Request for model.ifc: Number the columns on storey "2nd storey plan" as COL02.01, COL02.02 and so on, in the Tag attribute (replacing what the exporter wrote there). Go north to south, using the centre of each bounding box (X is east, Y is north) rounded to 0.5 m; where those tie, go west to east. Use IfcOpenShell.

First a look at what the model holds.

```python
import ifcopenshell
import ifcopenshell.util.element
import ifcopenshell.util.placement

model = ifcopenshell.open("model.ifc")
print(model.schema)
storey = next(s for s in model.by_type("IfcBuildingStorey") if s.Name == "2nd storey plan")
columns = [e for e in ifcopenshell.util.element.get_decomposition(storey) if e.is_a("IfcColumn")]
for e in sorted(columns, key=lambda e: e.id()):
    origin = ifcopenshell.util.placement.get_local_placement(e.ObjectPlacement)[:3, 3]
    print(e.id(), e.Tag, e.Name, origin.round(2) + 0.0, sep=" | ")
```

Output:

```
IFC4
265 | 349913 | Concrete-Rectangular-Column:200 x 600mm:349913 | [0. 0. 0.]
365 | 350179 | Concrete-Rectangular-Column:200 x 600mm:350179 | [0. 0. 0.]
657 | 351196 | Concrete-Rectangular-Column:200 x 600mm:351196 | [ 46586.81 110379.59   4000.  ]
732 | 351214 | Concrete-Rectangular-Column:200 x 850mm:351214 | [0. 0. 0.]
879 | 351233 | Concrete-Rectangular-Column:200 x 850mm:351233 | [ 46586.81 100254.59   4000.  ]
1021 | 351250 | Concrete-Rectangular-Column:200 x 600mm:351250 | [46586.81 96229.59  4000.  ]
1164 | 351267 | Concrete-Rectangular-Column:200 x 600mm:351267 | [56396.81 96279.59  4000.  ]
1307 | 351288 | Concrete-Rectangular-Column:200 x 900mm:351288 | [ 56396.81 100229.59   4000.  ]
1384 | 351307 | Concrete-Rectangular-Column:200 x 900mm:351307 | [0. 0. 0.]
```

```python
import ifcopenshell
import ifcopenshell.geom
import ifcopenshell.util.element
import ifcopenshell.util.shape

model = ifcopenshell.open("model.ifc")
settings = ifcopenshell.geom.settings()
settings.set("use-world-coords", True)


def centre(element):
    shape = ifcopenshell.geom.create_shape(settings, element)
    return ifcopenshell.util.shape.get_bbox_centroid(shape.geometry)


storey = next(s for s in model.by_type("IfcBuildingStorey") if s.Name == "2nd storey plan")
columns = [e for e in ifcopenshell.util.element.get_decomposition(storey) if e.is_a("IfcColumn")]

# Insertion points can sit at a corner or the storey origin, so sort by the geometry (in metres).
centres = {e: centre(e) for e in columns}
columns.sort(key=lambda e: (-round(centres[e][1] / 0.5), centres[e][0]))

for i, e in enumerate(columns, start=1):
    number = f"COL02.{i:02d}"
    e.Tag = number
    print(e.id(), number)

model.write("model_rev.ifc")
```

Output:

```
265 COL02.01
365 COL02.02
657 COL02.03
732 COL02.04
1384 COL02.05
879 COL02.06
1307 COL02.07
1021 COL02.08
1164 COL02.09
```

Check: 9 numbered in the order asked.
